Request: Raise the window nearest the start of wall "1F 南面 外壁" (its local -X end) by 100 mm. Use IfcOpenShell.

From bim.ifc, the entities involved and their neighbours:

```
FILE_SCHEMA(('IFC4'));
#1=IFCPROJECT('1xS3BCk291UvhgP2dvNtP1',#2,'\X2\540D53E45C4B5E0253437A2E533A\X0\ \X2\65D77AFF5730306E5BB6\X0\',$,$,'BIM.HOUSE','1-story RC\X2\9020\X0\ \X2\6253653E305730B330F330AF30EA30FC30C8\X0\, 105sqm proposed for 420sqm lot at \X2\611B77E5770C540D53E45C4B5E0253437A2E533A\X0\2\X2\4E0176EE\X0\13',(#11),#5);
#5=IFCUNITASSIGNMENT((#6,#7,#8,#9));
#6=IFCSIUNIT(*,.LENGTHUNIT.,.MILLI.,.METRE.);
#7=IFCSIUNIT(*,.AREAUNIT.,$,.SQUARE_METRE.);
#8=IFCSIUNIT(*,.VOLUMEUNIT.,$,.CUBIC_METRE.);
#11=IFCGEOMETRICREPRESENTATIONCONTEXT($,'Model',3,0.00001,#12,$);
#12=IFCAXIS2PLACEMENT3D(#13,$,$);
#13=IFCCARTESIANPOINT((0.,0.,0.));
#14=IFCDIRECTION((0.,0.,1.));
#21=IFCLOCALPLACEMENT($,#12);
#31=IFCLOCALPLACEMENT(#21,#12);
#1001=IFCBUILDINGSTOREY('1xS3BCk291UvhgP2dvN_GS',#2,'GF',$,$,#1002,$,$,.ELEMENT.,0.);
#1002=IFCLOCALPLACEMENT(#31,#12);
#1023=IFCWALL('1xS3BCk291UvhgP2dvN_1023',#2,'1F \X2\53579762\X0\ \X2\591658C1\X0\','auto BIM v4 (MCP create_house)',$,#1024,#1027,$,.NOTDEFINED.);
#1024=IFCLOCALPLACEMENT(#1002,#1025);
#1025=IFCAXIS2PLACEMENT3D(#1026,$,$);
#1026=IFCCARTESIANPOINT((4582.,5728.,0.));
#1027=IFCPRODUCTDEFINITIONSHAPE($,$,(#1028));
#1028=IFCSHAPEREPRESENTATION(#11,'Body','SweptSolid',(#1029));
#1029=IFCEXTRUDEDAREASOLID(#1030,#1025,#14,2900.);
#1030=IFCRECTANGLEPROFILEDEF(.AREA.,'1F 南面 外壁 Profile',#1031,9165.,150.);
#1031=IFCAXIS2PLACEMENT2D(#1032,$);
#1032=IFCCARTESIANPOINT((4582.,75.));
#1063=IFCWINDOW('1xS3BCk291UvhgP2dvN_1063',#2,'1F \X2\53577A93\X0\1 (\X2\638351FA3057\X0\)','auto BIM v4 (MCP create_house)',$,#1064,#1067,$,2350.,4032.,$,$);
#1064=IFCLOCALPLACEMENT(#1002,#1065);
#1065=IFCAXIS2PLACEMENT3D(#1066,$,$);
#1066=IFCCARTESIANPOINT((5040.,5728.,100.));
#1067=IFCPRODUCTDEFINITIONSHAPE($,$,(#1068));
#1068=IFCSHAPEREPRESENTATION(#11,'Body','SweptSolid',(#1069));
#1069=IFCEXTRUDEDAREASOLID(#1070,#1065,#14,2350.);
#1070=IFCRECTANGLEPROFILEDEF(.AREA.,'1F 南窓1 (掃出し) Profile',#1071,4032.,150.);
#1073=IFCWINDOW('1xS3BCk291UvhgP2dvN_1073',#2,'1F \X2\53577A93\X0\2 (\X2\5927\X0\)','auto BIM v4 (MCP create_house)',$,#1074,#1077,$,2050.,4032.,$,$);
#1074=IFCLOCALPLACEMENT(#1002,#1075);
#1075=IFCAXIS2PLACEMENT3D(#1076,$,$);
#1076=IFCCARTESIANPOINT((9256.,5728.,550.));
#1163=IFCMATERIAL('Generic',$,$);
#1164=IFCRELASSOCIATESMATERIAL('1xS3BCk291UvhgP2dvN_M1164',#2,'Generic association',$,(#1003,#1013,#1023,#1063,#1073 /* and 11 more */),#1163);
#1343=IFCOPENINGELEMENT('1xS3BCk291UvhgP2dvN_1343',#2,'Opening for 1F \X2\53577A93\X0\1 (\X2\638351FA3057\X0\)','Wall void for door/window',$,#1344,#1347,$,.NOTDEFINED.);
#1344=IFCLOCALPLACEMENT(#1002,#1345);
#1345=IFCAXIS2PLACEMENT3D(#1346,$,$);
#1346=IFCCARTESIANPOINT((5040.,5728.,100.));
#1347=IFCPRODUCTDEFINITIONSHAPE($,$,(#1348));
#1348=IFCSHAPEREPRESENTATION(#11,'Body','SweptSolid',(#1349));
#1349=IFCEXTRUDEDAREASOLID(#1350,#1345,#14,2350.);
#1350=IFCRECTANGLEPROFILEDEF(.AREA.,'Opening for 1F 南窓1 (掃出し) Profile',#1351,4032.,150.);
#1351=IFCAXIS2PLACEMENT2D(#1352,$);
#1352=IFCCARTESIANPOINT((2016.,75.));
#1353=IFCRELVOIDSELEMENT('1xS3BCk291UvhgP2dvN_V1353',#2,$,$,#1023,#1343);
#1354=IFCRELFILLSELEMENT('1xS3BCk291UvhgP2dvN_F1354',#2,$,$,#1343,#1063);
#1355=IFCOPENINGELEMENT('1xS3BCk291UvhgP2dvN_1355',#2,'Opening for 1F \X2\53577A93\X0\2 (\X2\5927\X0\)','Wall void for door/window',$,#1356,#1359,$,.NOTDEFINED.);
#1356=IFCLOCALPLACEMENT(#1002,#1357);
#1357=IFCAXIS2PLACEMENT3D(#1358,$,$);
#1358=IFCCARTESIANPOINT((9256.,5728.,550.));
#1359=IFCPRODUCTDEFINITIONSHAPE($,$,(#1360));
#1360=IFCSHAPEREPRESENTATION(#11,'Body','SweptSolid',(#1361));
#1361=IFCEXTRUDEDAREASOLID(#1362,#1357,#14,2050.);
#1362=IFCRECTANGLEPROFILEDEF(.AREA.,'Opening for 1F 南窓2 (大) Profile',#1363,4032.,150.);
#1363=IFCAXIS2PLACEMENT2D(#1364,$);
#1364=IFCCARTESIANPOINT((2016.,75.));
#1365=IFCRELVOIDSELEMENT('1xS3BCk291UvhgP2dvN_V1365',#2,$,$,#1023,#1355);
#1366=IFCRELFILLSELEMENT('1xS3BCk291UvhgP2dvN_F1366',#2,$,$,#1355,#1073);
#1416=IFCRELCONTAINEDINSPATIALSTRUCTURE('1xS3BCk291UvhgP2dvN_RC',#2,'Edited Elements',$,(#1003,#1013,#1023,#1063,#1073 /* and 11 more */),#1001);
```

```python
import numpy as np
import ifcopenshell
import ifcopenshell.api.geometry
import ifcopenshell.util.placement
import ifcopenshell.util.unit

model = ifcopenshell.open("bim.ifc")
unit_scale = ifcopenshell.util.unit.calculate_unit_scale(model)

window = model.by_guid("1xS3BCk291UvhgP2dvN_1063")
opening = window.FillsVoids[0].RelatingOpeningElement
dz = 0.1 / unit_scale

shift = np.array([0.0, 0.0, dz])
# The window is not placed relative to its opening, so move both.
for product in (opening, window):
    matrix = ifcopenshell.util.placement.get_local_placement(product.ObjectPlacement)
    matrix[:3, 3] += shift
    ifcopenshell.api.geometry.edit_object_placement(model, product=product, matrix=matrix, is_si=False)

print(f"moved by {dz * unit_scale:+.3f} m")

model.write("bim_rev.ifc")
```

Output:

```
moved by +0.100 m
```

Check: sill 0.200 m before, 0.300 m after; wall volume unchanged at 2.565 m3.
